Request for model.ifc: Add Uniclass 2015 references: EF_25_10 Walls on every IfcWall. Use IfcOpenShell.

First a look at what the model holds.

```python
import ifcopenshell

model = ifcopenshell.open("model.ifc")
print(model.schema)
print("classifications:", [c.Name for c in model.by_type("IfcClassification")])
for ifc_class in ("IfcDoor", "IfcRoof", "IfcStair", "IfcWall", "IfcWindow"):
    print(ifc_class, len(model.by_type(ifc_class)))
```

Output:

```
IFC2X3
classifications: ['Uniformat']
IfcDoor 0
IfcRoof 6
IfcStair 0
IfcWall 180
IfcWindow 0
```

```python
import ifcopenshell
import ifcopenshell.api.classification

model = ifcopenshell.open("model.ifc")

# IFC2X3 requires Source and Edition and has no link from the project to the system.
system = model.create_entity("IfcClassification", Source="NBS", Edition="2015", Name="Uniclass 2015")

codes = {
    "IfcWall": ("EF_25_10", "Walls"),
}
for ifc_class, (code, name) in codes.items():
    products = model.by_type(ifc_class)
    ifcopenshell.api.classification.add_reference(
        model, products=products, classification=system, identification=code, name=name
    )
    print(code, len(products))

model.write("model_edited.ifc")
```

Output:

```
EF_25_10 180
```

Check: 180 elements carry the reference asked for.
